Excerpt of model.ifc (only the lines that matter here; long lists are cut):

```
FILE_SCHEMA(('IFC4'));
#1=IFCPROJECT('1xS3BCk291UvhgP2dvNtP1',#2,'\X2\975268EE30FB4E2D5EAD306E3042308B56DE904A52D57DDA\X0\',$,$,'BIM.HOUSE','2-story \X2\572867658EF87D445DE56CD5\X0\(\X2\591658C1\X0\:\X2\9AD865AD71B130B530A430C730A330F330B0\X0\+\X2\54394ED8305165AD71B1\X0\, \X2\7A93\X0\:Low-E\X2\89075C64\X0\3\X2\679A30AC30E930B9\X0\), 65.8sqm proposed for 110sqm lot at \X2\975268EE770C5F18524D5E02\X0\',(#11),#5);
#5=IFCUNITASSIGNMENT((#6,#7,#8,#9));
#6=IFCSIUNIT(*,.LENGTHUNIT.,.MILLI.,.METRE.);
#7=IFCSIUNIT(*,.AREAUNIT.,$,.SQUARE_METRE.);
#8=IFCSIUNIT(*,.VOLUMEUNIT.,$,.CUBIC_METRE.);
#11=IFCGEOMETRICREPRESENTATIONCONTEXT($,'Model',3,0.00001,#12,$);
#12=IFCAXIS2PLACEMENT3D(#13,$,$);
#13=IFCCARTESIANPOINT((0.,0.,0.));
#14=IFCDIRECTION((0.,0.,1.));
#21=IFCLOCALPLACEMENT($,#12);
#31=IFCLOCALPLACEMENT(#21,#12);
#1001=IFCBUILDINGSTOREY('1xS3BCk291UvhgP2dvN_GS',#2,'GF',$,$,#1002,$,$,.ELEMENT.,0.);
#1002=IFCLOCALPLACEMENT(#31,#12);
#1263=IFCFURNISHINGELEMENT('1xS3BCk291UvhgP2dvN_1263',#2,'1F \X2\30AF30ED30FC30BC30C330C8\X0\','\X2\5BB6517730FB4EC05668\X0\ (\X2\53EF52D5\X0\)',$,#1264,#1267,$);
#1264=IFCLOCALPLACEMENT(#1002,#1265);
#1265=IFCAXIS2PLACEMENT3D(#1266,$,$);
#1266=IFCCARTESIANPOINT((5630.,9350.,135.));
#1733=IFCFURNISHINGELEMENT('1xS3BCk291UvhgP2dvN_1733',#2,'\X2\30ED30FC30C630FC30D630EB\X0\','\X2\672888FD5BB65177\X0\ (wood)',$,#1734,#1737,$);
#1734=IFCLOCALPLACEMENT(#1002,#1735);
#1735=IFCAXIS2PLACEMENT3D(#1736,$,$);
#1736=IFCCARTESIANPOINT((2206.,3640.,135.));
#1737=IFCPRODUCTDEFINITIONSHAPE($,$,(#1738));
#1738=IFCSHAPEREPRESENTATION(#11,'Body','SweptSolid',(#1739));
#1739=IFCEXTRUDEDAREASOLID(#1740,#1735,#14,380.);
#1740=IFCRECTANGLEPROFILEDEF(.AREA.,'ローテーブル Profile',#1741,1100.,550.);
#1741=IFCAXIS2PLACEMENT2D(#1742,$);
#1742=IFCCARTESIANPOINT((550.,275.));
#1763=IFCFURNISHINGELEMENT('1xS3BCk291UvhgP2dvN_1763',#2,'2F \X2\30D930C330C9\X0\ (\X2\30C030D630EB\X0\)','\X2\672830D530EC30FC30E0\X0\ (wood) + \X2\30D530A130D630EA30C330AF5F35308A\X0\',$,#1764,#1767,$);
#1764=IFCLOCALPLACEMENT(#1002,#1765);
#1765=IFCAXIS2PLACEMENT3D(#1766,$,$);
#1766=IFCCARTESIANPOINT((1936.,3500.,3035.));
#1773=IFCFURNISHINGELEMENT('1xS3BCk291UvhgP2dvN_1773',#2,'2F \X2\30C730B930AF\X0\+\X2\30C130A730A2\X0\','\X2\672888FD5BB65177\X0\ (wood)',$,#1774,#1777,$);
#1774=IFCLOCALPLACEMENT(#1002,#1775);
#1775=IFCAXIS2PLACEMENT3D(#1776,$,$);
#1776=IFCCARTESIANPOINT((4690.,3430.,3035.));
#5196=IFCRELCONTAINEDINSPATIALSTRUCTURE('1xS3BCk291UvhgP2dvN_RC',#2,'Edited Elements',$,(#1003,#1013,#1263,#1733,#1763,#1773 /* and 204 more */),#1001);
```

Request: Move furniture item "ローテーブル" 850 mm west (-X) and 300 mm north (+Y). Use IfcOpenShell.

```python
import ifcopenshell
import ifcopenshell.api.geometry
import ifcopenshell.util.placement

model = ifcopenshell.open("model.ifc")

item = model.by_id(1733)
matrix = ifcopenshell.util.placement.get_local_placement(item.ObjectPlacement)
matrix[0, 3] -= 850.0
matrix[1, 3] += 300.0
ifcopenshell.api.geometry.edit_object_placement(model, product=item, matrix=matrix, is_si=False)

print(ifcopenshell.util.placement.get_local_placement(item.ObjectPlacement).round(3) + 0.0)

model.write("model-out.ifc")
```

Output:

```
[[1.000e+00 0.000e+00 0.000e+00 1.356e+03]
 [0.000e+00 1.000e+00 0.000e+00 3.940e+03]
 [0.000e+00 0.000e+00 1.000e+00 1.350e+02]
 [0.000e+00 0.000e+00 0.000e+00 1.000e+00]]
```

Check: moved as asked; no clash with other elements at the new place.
